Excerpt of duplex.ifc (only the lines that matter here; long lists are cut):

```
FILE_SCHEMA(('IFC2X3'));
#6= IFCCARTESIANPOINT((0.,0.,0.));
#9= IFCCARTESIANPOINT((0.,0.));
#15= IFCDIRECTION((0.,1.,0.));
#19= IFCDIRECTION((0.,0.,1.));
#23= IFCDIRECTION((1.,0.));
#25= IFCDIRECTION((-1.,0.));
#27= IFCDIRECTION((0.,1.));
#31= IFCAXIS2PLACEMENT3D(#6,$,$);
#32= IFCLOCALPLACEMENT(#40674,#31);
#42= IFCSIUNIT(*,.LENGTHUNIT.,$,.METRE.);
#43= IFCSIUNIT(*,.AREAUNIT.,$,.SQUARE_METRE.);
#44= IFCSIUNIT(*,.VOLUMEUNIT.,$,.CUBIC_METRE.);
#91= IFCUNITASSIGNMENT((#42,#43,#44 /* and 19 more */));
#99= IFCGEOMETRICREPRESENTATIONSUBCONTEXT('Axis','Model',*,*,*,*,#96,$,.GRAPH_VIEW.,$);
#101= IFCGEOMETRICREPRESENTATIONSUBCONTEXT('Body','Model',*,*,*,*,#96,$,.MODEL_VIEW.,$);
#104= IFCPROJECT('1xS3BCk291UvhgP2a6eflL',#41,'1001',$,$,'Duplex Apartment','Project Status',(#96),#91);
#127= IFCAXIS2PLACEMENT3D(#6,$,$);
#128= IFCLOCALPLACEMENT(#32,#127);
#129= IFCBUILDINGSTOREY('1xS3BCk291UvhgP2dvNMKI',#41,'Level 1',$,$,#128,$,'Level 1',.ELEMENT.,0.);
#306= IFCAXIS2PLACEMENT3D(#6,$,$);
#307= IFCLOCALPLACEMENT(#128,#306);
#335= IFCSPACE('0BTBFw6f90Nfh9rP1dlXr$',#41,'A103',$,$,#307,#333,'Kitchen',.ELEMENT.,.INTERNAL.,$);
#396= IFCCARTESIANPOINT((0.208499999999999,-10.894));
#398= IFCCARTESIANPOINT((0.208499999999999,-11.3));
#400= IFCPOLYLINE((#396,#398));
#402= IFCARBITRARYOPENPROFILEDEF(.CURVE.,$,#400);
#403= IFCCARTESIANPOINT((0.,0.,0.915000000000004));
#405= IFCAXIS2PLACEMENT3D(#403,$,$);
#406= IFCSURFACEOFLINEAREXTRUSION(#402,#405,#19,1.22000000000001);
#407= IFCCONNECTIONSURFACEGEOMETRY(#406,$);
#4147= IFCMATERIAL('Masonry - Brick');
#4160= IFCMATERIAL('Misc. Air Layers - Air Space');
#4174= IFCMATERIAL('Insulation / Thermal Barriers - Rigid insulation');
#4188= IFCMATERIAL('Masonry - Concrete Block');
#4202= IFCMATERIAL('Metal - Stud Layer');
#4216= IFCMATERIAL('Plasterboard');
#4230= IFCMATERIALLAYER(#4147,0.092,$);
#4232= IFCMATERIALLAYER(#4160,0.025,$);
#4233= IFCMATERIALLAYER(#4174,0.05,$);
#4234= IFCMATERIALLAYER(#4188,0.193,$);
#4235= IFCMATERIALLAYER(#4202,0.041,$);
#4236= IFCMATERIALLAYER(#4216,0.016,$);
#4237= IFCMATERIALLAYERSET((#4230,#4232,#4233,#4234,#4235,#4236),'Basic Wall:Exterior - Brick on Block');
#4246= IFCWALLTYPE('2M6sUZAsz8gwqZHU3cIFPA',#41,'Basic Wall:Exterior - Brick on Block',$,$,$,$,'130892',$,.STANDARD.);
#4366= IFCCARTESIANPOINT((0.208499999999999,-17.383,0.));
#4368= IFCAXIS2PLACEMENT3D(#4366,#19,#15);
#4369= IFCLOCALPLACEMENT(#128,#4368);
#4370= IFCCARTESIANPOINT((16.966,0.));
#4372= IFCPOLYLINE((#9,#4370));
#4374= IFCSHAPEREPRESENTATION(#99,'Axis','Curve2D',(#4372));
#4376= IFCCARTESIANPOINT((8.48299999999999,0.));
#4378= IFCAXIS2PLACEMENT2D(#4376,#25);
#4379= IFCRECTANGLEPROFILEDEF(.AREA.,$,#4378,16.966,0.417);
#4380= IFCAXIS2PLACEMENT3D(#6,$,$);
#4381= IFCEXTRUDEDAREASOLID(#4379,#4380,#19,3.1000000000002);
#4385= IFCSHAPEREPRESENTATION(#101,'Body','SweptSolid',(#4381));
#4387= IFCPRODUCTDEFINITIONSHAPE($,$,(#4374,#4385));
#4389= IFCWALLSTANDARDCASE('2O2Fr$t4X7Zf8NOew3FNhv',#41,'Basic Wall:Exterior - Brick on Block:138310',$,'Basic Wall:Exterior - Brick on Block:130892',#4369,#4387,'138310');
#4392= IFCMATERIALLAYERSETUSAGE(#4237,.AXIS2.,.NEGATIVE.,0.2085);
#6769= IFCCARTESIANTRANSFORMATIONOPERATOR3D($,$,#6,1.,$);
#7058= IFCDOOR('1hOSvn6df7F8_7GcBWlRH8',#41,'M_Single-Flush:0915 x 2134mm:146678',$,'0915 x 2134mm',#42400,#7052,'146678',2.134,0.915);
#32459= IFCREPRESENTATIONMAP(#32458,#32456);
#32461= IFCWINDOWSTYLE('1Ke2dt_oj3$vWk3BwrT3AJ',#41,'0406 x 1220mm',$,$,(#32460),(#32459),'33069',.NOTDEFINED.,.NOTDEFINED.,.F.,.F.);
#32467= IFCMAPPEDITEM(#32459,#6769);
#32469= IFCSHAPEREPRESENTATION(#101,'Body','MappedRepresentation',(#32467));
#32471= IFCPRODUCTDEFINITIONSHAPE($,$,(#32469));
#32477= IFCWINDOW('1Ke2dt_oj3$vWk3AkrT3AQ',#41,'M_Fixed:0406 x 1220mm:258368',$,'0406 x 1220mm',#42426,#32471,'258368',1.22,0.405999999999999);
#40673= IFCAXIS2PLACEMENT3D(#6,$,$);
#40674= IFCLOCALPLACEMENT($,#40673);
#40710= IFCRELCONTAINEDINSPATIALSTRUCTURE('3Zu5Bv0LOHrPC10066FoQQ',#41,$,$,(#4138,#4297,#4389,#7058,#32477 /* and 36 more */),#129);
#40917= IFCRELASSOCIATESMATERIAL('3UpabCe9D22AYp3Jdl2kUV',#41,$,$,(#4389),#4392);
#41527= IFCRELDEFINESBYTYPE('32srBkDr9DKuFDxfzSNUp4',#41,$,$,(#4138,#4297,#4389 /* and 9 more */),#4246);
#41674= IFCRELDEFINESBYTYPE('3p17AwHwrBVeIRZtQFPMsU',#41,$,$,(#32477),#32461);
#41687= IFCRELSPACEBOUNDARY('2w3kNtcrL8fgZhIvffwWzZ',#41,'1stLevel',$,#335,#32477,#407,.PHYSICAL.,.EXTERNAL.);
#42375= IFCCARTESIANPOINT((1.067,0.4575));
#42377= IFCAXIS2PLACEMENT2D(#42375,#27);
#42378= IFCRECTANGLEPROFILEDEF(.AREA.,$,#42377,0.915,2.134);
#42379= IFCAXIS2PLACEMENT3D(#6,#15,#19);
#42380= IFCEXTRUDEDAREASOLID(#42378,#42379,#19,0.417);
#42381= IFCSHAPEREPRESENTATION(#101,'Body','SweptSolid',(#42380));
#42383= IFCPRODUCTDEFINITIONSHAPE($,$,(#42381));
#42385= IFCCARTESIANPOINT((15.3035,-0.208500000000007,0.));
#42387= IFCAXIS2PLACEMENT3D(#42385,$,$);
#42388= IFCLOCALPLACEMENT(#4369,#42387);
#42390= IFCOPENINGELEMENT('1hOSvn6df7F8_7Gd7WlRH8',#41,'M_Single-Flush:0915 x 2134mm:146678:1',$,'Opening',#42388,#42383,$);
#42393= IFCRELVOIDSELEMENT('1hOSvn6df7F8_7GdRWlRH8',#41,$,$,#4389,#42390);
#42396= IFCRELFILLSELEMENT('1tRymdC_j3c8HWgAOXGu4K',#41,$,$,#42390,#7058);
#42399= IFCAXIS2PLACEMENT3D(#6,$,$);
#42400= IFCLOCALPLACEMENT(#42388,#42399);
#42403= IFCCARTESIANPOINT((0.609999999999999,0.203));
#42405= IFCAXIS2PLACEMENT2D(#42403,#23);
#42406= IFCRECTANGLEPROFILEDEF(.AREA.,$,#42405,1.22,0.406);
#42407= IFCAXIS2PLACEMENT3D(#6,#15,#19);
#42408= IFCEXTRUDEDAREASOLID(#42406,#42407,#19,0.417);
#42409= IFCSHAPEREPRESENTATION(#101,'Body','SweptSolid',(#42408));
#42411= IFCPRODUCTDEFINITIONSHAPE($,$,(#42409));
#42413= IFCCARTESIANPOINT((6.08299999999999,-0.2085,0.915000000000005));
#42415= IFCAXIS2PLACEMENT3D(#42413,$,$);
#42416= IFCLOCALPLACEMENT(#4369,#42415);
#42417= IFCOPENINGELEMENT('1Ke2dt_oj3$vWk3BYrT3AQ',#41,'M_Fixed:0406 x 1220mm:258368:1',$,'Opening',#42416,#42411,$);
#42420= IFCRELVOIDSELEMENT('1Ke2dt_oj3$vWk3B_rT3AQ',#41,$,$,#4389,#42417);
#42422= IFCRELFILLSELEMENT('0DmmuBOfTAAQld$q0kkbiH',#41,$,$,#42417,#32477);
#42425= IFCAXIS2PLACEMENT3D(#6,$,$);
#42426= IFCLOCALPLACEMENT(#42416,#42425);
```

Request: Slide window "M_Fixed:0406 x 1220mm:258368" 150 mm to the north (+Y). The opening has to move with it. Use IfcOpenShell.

```python
import numpy as np
import ifcopenshell
import ifcopenshell.api.geometry
import ifcopenshell.util.placement
import ifcopenshell.util.unit

model = ifcopenshell.open("duplex.ifc")
unit_scale = ifcopenshell.util.unit.calculate_unit_scale(model)

window = model.by_id(32477)
opening = window.FillsVoids[0].RelatingOpeningElement
wall = opening.VoidsElements[0].RelatingBuildingElement

wall_matrix = ifcopenshell.util.placement.get_local_placement(wall.ObjectPlacement)
shift = wall_matrix[:3, 0] * 0.15 / unit_scale
before = ifcopenshell.util.placement.get_local_placement(window.ObjectPlacement)[:3, 3].copy()

# The window is placed relative to its opening, so it follows when the opening moves.
matrix = ifcopenshell.util.placement.get_local_placement(opening.ObjectPlacement)
matrix[:3, 3] += shift
ifcopenshell.api.geometry.edit_object_placement(
    model, product=opening, matrix=matrix, is_si=False, should_transform_children=True
)

# Space boundary surfaces are stored in each space's coordinates; move them too.
for rel in window.ProvidesBoundaries:
    if not rel.ConnectionGeometry:
        continue
    surface = rel.ConnectionGeometry.SurfaceOnRelatingElement
    space_matrix = ifcopenshell.util.placement.get_local_placement(rel.RelatingSpace.ObjectPlacement)
    point = np.array(surface.Position.Location.Coordinates) + space_matrix[:3, :3].T @ shift
    surface.Position = model.createIfcAxis2Placement3D(
        model.createIfcCartesianPoint(point.tolist()), surface.Position.Axis, surface.Position.RefDirection
    )

after = ifcopenshell.util.placement.get_local_placement(window.ObjectPlacement)[:3, 3]
print("window moved by", (after - before).round(3) + 0.0)

model.write("duplex_rev.ifc")
```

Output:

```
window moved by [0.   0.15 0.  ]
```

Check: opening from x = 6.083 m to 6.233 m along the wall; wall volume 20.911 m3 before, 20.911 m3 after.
